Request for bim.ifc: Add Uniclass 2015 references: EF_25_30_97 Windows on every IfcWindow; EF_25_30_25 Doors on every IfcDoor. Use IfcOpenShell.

First a look at what the model holds.

```python
import ifcopenshell

model = ifcopenshell.open("bim.ifc")
print(model.schema)
print("classifications:", [c.Name for c in model.by_type("IfcClassification")])
for ifc_class in ("IfcDoor", "IfcRoof", "IfcStair", "IfcWall", "IfcWindow"):
    print(ifc_class, len(model.by_type(ifc_class)))
```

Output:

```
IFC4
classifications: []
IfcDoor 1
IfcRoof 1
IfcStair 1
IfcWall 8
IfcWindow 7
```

```python
import ifcopenshell
import ifcopenshell.api.classification

model = ifcopenshell.open("bim.ifc")

system = ifcopenshell.api.classification.add_classification(model, classification="Uniclass 2015")

codes = {
    "IfcWindow": ("EF_25_30_97", "Windows"),
    "IfcDoor": ("EF_25_30_25", "Doors"),
}
for ifc_class, (code, name) in codes.items():
    products = model.by_type(ifc_class)
    ifcopenshell.api.classification.add_reference(
        model, products=products, classification=system, identification=code, name=name
    )
    print(code, len(products))

model.write("bim_v2.ifc")
```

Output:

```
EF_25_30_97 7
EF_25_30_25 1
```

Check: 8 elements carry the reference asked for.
